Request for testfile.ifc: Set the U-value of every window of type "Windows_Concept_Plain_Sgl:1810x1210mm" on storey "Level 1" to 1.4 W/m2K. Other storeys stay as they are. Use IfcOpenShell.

First a look at what the model holds.

```python
import ifcopenshell
import ifcopenshell.util.element

model = ifcopenshell.open("testfile.ifc")
print(model.schema)
storey = next(s for s in model.by_type("IfcBuildingStorey") if s.Name == "Level 1")
windows = [e for e in ifcopenshell.util.element.get_decomposition(storey) if e.is_a("IfcWindow")]
seen = {}
for e in windows:
    element_type = ifcopenshell.util.element.get_type(e)
    key = (element_type.Name if element_type != e and element_type else None, ifcopenshell.util.element.get_pset(e, "Pset_WindowCommon", "ThermalTransmittance"))
    seen[key] = seen.get(key, 0) + 1
for (name, value), count in sorted(seen.items(), key=str):
    print(count, "x", name, "|", value)
```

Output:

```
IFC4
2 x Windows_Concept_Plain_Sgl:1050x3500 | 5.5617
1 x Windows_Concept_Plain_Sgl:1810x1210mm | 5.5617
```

```python
import ifcopenshell
import ifcopenshell.api.pset
import ifcopenshell.util.element

model = ifcopenshell.open("testfile.ifc")

storey = next(s for s in model.by_type("IfcBuildingStorey") if s.Name == "Level 1")
windows = [e for e in ifcopenshell.util.element.get_decomposition(storey) if e.is_a("IfcWindow")]

count = 0
for e in windows:
    element_type = ifcopenshell.util.element.get_type(e)
    if element_type in (None, e) or element_type.Name != "Windows_Concept_Plain_Sgl:1810x1210mm":
        continue
    # add_pset returns the element's existing set when there is one.
    pset = ifcopenshell.api.pset.add_pset(model, product=e, name="Pset_WindowCommon")
    ifcopenshell.api.pset.edit_pset(model, pset=pset, properties={"ThermalTransmittance": 1.4})
    count += 1

print(count, "windows updated")

model.write("testfile_rev.ifc")
```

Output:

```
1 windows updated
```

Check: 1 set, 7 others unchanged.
